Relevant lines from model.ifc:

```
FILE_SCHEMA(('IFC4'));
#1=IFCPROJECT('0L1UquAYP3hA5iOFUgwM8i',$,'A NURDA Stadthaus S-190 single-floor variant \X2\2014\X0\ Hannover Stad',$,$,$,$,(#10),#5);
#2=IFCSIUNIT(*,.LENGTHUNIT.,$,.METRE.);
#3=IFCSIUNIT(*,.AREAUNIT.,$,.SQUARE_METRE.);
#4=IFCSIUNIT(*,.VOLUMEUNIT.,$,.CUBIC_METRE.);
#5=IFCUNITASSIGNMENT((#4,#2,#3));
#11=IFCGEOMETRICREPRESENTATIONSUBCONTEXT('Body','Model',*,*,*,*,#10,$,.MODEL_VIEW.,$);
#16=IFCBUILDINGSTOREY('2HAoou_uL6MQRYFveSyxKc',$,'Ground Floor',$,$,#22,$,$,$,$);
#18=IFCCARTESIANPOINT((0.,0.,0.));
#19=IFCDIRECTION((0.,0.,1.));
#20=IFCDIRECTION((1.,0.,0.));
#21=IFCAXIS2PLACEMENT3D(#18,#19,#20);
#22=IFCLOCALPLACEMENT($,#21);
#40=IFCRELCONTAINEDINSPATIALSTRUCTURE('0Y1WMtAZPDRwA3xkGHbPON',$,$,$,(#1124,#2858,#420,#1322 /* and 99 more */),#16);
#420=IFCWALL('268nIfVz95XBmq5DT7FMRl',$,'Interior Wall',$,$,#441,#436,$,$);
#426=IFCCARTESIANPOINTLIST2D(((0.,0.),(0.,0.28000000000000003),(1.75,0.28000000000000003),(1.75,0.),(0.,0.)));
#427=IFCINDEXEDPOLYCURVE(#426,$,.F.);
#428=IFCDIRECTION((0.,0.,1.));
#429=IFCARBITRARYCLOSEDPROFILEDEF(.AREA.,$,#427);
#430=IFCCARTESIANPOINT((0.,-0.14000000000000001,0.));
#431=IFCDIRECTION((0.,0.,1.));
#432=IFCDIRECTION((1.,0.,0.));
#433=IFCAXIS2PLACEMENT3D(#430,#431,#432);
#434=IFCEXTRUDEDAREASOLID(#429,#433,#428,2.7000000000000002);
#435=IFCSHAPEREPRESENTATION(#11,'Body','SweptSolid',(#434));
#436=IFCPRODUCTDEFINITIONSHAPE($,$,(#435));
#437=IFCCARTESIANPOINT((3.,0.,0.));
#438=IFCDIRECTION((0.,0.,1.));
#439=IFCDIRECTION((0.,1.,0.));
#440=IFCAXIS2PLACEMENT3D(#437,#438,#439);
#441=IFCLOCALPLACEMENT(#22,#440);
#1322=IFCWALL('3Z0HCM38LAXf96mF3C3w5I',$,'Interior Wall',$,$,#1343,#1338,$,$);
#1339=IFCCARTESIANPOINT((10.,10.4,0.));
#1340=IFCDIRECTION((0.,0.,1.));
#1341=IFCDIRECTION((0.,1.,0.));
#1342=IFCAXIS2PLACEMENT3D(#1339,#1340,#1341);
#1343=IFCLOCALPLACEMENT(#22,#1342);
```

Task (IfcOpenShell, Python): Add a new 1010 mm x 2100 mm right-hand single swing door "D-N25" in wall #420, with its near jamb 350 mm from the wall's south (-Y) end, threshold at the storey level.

```python
import numpy as np
import ifcopenshell
import ifcopenshell.api.feature
import ifcopenshell.api.geometry
import ifcopenshell.api.root
import ifcopenshell.api.spatial
import ifcopenshell.geom
import ifcopenshell.util.element
import ifcopenshell.util.placement
import ifcopenshell.util.representation
import ifcopenshell.util.shape
import ifcopenshell.util.unit

model = ifcopenshell.open("model.ifc")
unit_scale = ifcopenshell.util.unit.calculate_unit_scale(model)
settings = ifcopenshell.geom.settings()


def volume(element):
    """Net volume in cubic metres, openings subtracted."""
    shape = ifcopenshell.geom.create_shape(settings, element)
    return ifcopenshell.util.shape.get_volume(shape.geometry)


wall = model.by_guid("268nIfVz95XBmq5DT7FMRl")
storey = ifcopenshell.util.element.get_container(wall, ifc_class="IfcBuildingStorey")
context = ifcopenshell.util.representation.get_context(model, "Model", "Body", "MODEL_VIEW")
before = volume(wall)

width, height, from_end, sill = 1.01, 2.1, 0.35, 0.0  # metres

# The wall runs along its own X axis, and the end named is its -X end.
wall_shape = ifcopenshell.geom.create_shape(settings, wall)
x, y, z = ifcopenshell.util.shape.get_vertices(wall_shape.geometry).T
start = x.min() + from_end
face, thickness = float(y.min()), float(y.max() - y.min())
wall_matrix = ifcopenshell.util.placement.get_local_placement(wall.ObjectPlacement)
level = ifcopenshell.util.placement.get_local_placement(storey.ObjectPlacement)[2, 3]


def in_wall(x, y):
    """Placement at x, y metres in the wall's axes, at sill height."""
    matrix = wall_matrix.copy()
    matrix[:, 3] = wall_matrix @ np.array([x / unit_scale, y / unit_scale, 0.0, 1.0])
    matrix[2, 3] = level + sill / unit_scale
    return matrix


# Opening: a box that overshoots both wall faces by 50 mm.
opening = ifcopenshell.api.root.create_entity(model, ifc_class="IfcOpeningElement", predefined_type="OPENING")
box = ifcopenshell.api.geometry.add_wall_representation(
    model, context=context, length=width, height=height, thickness=thickness + 0.1
)
ifcopenshell.api.geometry.assign_representation(model, product=opening, representation=box)
ifcopenshell.api.geometry.edit_object_placement(model, product=opening, matrix=in_wall(start, face - 0.05), is_si=False)
ifcopenshell.api.feature.add_feature(model, feature=opening, element=wall)

door = ifcopenshell.api.root.create_entity(model, ifc_class="IfcDoor", name="D-N25", predefined_type="DOOR")
door.OverallWidth, door.OverallHeight = width / unit_scale, height / unit_scale
door.OperationType = "SINGLE_SWING_RIGHT"
body = ifcopenshell.api.geometry.add_door_representation(
    model,
    context=context,
    overall_width=door.OverallWidth,
    overall_height=door.OverallHeight,
    operation_type="SINGLE_SWING_RIGHT",
    lining_properties={"LiningDepth": thickness / unit_scale, "ThresholdDepth": thickness / unit_scale},
)
ifcopenshell.api.geometry.assign_representation(model, product=door, representation=body)
ifcopenshell.api.spatial.assign_container(model, products=[door], relating_structure=storey)
ifcopenshell.api.feature.add_filling(model, opening=opening, element=door)

# The lining spans the wall, so the door starts at the wall face.
ifcopenshell.api.geometry.edit_object_placement(model, product=door, matrix=in_wall(start, face), is_si=False)

after = volume(wall)

print(f"wall volume {before:.3f} -> {after:.3f} m3")

model.write("model_updated.ifc")
```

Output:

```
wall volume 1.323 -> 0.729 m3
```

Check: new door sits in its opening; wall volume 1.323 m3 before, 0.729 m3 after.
